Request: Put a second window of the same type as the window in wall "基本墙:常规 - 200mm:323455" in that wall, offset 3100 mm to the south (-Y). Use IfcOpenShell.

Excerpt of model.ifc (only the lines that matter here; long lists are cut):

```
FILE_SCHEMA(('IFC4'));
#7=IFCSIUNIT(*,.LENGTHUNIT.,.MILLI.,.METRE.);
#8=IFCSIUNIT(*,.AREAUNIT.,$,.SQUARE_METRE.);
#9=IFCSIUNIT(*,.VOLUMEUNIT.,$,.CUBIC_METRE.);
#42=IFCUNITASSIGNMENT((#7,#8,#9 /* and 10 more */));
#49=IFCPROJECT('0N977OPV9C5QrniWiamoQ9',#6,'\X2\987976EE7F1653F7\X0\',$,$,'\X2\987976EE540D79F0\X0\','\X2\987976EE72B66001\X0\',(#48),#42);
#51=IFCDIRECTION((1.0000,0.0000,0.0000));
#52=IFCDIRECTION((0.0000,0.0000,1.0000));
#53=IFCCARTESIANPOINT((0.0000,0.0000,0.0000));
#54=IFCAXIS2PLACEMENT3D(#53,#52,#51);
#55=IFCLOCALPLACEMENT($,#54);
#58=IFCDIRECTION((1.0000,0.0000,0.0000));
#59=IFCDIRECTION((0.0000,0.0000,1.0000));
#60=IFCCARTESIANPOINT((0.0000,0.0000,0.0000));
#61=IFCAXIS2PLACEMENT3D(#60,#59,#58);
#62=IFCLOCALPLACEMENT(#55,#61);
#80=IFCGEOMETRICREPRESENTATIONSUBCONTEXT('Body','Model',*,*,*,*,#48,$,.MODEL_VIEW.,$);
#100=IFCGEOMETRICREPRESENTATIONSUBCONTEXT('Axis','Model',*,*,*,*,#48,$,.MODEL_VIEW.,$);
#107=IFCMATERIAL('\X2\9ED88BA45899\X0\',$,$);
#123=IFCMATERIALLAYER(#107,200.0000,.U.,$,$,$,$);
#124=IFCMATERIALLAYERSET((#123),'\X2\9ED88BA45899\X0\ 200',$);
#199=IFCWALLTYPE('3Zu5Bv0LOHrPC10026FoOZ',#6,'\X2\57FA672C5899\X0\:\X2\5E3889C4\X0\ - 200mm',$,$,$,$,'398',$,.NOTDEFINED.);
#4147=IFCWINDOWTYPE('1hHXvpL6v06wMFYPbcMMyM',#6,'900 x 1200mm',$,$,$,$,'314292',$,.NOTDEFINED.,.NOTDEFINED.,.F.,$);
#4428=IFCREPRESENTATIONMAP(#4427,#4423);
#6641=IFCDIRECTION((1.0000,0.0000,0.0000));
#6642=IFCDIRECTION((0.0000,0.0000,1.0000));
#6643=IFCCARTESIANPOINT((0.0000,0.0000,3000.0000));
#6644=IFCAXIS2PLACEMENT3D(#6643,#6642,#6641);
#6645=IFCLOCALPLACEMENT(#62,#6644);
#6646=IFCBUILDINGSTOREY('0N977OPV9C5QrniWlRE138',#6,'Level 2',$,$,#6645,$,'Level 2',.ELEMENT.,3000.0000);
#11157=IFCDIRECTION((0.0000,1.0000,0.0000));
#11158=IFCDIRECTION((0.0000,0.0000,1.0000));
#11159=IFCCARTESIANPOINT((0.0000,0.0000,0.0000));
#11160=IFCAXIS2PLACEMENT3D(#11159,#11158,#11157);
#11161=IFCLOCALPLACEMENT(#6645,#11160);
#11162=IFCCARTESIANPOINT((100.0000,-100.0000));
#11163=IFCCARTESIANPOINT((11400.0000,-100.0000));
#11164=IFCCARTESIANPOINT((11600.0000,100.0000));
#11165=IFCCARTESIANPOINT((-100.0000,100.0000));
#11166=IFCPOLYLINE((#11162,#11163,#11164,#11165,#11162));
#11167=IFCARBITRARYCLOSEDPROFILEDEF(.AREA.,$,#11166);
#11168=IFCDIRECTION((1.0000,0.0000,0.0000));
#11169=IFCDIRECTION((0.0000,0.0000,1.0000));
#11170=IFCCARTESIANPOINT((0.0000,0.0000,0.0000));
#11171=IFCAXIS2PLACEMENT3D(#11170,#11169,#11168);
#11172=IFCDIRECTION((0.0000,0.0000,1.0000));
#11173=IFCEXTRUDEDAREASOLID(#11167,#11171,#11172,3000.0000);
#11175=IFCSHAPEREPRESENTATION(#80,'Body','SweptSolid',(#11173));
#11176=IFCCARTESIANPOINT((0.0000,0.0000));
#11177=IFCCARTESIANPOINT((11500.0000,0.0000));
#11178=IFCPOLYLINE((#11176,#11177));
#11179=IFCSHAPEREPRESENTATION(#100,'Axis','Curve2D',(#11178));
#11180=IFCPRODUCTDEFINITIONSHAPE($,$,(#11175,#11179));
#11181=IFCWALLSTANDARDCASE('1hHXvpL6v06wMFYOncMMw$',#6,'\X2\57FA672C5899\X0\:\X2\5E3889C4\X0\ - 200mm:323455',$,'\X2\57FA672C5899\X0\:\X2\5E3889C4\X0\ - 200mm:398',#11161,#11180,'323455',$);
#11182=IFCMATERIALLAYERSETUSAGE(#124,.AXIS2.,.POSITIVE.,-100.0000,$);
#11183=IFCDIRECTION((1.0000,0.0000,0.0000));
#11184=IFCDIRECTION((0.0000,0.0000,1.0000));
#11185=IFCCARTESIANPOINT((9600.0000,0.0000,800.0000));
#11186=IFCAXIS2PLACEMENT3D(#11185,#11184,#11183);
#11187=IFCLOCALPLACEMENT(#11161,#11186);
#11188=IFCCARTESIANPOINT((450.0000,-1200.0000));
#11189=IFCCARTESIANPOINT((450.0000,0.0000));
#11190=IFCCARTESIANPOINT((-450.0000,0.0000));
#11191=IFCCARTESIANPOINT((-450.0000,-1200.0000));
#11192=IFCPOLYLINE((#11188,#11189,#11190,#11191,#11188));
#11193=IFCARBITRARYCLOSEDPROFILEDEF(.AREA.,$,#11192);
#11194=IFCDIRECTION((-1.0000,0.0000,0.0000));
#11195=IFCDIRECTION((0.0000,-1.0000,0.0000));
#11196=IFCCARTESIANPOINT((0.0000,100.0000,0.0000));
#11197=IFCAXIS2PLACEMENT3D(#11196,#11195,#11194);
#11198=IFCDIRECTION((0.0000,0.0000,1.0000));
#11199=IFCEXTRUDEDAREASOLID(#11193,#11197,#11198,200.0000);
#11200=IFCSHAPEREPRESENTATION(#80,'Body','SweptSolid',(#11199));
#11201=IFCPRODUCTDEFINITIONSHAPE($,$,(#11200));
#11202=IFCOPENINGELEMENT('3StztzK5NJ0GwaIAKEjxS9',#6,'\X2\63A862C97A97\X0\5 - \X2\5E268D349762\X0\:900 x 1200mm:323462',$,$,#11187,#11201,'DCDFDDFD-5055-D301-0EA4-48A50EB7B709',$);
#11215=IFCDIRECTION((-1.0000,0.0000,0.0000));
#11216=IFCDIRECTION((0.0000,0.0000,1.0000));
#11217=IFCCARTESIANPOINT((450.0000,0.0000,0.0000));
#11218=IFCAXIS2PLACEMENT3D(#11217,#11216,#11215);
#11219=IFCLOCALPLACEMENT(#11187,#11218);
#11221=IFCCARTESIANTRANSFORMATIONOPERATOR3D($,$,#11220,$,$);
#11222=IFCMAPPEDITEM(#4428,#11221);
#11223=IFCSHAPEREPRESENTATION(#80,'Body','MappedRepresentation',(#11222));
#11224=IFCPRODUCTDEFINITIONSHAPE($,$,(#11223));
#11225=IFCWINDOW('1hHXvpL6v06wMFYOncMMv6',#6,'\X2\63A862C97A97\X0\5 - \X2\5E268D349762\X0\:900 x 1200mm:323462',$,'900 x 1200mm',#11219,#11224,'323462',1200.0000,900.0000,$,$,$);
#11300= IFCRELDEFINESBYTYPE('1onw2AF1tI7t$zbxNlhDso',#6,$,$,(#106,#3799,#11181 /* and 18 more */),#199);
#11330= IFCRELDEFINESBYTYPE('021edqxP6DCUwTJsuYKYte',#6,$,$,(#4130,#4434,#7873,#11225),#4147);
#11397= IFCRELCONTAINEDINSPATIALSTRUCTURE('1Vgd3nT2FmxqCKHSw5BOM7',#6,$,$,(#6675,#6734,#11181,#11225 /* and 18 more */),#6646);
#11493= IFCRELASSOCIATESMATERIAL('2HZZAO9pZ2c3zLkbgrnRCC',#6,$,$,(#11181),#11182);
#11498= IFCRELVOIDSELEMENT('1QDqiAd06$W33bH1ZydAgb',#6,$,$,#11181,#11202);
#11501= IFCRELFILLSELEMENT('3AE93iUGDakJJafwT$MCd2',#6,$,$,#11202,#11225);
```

```python
import ifcopenshell
import ifcopenshell.api.feature
import ifcopenshell.api.geometry
import ifcopenshell.api.root
import ifcopenshell.geom
import ifcopenshell.util.element
import ifcopenshell.util.placement
import ifcopenshell.util.shape
import ifcopenshell.util.unit

model = ifcopenshell.open("model.ifc")
unit_scale = ifcopenshell.util.unit.calculate_unit_scale(model)
settings = ifcopenshell.geom.settings()


def volume(element):
    """Net volume in cubic metres, openings subtracted."""
    shape = ifcopenshell.geom.create_shape(settings, element)
    return ifcopenshell.util.shape.get_volume(shape.geometry)


def reuse_history(source, copy):
    """copy_class also copies each property set's owner history, people and application; keep the originals."""
    for rel in copy.IsDefinedBy:
        if rel.is_a("IfcRelDefinesByProperties") and (history := rel.RelatingPropertyDefinition.OwnerHistory):
            rel.RelatingPropertyDefinition.OwnerHistory = source.OwnerHistory
            ifcopenshell.util.element.remove_deep2(model, history)


window = model.by_guid("1hHXvpL6v06wMFYOncMMv6")
opening = window.FillsVoids[0].RelatingOpeningElement
wall = opening.VoidsElements[0].RelatingBuildingElement
before = volume(wall)
shift = ifcopenshell.util.placement.get_local_placement(wall.ObjectPlacement)[:3, 0] * -3.1 / unit_scale

# copy_class copies the void relationship, type, container and properties, but no geometry.
new_opening = ifcopenshell.api.root.copy_class(model, product=opening)
new_opening.Representation = ifcopenshell.util.element.copy_deep(
    model, opening.Representation, exclude=["IfcGeometricRepresentationContext", "IfcRepresentationMap"]
)
new_opening.Name = "推拉窗5 - 带贴面:900 x 1200mm"
new_opening.Tag = None
new_window = ifcopenshell.api.root.copy_class(model, product=window)
new_window.Representation = ifcopenshell.util.element.copy_deep(
    model, window.Representation, exclude=["IfcGeometricRepresentationContext", "IfcRepresentationMap"]
)
new_window.Name = "推拉窗5 - 带贴面:900 x 1200mm"
new_window.Tag = None
reuse_history(window, new_window)
ifcopenshell.api.feature.add_filling(model, opening=new_opening, element=new_window)

for old, new in ((opening, new_opening), (window, new_window)):
    matrix = ifcopenshell.util.placement.get_local_placement(old.ObjectPlacement)
    matrix[:3, 3] += shift
    ifcopenshell.api.geometry.edit_object_placement(model, product=new, matrix=matrix, is_si=False)

after = volume(wall)

print(f"wall volume {before:.3f} -> {after:.3f} m3")

model.write("model_v2.ifc")
```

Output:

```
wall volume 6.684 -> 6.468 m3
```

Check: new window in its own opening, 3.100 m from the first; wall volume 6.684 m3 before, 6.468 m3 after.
